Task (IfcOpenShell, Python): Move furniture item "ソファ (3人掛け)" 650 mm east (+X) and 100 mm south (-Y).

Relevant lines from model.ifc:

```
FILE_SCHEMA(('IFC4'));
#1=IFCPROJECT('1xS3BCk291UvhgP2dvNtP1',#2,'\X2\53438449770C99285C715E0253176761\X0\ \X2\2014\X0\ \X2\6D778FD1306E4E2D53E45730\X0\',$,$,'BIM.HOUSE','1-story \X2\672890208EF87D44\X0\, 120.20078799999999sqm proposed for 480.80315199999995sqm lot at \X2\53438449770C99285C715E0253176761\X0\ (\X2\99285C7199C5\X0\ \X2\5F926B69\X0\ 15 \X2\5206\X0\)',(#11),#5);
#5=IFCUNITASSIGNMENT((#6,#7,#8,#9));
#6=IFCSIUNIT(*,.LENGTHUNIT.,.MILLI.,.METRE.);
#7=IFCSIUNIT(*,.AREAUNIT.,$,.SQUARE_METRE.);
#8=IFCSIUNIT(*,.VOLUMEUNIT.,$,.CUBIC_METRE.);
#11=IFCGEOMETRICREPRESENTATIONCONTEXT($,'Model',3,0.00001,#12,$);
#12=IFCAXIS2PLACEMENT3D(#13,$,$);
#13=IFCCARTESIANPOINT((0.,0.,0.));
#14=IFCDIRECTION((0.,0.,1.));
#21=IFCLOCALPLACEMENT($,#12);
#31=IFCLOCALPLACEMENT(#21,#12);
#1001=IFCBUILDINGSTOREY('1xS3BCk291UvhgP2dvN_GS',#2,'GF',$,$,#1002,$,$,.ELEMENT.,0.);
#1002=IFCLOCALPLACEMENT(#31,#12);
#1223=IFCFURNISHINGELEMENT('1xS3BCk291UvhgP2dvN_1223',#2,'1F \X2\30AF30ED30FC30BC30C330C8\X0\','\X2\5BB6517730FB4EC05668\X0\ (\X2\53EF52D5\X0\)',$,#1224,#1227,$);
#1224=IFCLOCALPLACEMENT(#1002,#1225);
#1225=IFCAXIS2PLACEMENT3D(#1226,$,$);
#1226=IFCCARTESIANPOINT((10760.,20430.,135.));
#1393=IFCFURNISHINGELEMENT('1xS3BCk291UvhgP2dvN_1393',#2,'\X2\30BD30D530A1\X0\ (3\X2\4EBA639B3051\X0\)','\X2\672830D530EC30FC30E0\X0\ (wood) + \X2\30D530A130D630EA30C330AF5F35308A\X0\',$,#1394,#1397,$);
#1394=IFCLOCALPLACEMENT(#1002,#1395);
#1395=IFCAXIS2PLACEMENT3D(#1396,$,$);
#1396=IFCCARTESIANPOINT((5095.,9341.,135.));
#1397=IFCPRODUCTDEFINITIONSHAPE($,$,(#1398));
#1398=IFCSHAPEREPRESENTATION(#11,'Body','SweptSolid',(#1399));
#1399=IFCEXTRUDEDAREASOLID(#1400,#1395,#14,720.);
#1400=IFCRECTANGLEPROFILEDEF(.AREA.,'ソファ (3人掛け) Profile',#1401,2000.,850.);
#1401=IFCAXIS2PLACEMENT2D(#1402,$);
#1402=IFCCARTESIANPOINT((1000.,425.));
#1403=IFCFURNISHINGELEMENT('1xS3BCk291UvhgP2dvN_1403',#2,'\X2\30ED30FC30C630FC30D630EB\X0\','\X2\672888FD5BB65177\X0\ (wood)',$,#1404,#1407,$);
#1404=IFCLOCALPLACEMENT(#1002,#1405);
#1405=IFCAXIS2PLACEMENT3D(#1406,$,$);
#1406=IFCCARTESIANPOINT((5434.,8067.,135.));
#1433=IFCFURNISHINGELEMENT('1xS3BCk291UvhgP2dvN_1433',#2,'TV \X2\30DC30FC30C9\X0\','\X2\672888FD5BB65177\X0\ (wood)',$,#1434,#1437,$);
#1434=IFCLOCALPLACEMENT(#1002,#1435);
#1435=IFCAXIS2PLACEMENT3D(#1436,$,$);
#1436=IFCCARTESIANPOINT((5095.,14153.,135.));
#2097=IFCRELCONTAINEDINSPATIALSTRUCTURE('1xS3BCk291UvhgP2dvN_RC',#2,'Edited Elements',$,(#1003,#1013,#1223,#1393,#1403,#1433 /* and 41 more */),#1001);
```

```python
import ifcopenshell
import ifcopenshell.api.geometry
import ifcopenshell.util.placement
import ifcopenshell.util.unit

model = ifcopenshell.open("model.ifc")
unit_scale = ifcopenshell.util.unit.calculate_unit_scale(model)

item = model.by_guid("1xS3BCk291UvhgP2dvN_1393")
matrix = ifcopenshell.util.placement.get_local_placement(item.ObjectPlacement)
matrix[0, 3] += 0.65 / unit_scale
matrix[1, 3] -= 0.1 / unit_scale
ifcopenshell.api.geometry.edit_object_placement(model, product=item, matrix=matrix, is_si=False)

print(ifcopenshell.util.placement.get_local_placement(item.ObjectPlacement).round(3) + 0.0)

model.write("model_updated.ifc")
```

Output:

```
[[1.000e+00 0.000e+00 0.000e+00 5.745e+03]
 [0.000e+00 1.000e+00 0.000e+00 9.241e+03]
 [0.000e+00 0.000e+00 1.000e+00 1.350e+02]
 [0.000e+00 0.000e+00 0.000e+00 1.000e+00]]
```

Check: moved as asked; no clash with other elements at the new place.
